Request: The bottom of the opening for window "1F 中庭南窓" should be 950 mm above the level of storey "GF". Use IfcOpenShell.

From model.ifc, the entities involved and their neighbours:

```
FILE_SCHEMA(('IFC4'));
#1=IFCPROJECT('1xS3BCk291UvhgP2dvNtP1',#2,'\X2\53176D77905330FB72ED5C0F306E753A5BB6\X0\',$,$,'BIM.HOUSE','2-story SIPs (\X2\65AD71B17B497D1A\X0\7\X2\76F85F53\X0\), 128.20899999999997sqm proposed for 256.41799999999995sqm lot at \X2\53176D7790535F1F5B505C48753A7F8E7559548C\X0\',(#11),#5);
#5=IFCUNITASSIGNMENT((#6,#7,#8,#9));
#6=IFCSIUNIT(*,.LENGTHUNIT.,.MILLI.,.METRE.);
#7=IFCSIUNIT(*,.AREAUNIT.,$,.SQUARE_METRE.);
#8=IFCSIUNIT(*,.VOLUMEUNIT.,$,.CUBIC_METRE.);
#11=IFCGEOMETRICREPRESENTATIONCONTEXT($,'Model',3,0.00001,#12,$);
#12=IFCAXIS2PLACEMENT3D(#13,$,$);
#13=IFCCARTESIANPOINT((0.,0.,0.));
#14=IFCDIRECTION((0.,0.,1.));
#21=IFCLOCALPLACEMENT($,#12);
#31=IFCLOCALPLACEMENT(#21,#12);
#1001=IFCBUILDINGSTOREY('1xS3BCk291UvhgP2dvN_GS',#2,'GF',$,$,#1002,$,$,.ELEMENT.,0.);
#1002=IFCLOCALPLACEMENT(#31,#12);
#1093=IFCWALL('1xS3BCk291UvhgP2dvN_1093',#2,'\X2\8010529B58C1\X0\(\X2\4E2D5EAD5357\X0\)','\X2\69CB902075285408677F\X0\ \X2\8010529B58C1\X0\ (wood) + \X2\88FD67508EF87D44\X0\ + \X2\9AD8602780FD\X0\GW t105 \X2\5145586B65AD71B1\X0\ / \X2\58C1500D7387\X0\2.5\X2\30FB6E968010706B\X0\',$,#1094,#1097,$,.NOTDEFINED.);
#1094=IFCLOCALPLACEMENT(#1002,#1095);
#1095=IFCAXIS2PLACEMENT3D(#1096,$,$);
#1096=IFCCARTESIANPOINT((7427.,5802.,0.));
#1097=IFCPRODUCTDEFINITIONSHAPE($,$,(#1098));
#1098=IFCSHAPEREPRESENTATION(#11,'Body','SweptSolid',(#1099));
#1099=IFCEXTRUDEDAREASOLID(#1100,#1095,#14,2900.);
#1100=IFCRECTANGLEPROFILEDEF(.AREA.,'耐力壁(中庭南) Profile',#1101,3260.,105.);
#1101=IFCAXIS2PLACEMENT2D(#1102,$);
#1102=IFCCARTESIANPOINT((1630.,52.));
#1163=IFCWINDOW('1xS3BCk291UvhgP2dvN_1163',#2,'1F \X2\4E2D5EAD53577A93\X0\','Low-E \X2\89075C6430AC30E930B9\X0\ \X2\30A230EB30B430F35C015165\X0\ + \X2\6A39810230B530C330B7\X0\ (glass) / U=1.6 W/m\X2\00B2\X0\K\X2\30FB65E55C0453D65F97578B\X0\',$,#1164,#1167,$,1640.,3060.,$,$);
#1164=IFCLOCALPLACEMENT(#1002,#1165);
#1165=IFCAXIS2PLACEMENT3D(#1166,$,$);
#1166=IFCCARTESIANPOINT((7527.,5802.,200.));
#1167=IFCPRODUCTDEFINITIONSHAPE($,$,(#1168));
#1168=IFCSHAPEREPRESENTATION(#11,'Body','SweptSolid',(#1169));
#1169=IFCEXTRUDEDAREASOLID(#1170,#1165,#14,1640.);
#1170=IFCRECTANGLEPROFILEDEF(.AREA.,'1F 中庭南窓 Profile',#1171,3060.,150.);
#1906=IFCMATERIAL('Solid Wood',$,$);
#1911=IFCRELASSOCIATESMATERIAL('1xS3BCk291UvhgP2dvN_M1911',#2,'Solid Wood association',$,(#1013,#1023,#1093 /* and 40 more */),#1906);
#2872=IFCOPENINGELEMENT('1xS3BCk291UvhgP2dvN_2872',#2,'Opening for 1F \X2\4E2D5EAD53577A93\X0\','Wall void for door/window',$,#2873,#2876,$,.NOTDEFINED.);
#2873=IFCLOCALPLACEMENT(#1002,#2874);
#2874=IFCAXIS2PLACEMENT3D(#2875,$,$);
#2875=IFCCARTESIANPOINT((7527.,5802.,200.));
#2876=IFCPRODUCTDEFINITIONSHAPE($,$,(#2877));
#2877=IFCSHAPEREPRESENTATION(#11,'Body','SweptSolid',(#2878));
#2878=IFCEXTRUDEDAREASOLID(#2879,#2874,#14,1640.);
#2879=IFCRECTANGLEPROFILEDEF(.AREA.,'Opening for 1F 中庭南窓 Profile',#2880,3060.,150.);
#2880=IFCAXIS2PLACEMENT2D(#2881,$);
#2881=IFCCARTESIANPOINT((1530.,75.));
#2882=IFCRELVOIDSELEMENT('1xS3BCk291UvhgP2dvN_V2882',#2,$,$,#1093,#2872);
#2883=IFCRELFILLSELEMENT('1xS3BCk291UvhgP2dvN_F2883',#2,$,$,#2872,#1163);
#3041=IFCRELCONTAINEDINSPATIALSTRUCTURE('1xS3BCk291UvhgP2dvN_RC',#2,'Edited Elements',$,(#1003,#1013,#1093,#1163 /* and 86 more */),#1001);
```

```python
import numpy as np
import ifcopenshell
import ifcopenshell.api.geometry
import ifcopenshell.geom
import ifcopenshell.util.element
import ifcopenshell.util.placement
import ifcopenshell.util.shape
import ifcopenshell.util.unit

model = ifcopenshell.open("model.ifc")
unit_scale = ifcopenshell.util.unit.calculate_unit_scale(model)

window = model.by_guid("1xS3BCk291UvhgP2dvN_1163")
opening = window.FillsVoids[0].RelatingOpeningElement
storey = ifcopenshell.util.element.get_container(window, ifc_class="IfcBuildingStorey")
level = ifcopenshell.util.placement.get_local_placement(storey.ObjectPlacement)[2, 3]

# The opening's origin need not be at the sill, so measure its lowest point.
shape = ifcopenshell.geom.create_shape(ifcopenshell.geom.settings(), opening)
bottom = ifcopenshell.util.shape.get_shape_bottom_elevation(shape, shape.geometry) / unit_scale
dz = level + 0.95 / unit_scale - bottom

shift = np.array([0.0, 0.0, dz])
# The window is not placed relative to its opening, so move both.
for product in (opening, window):
    matrix = ifcopenshell.util.placement.get_local_placement(product.ObjectPlacement)
    matrix[:3, 3] += shift
    ifcopenshell.api.geometry.edit_object_placement(model, product=product, matrix=matrix, is_si=False)

print(f"moved by {dz * unit_scale:+.3f} m")

model.write("model_v2.ifc")
```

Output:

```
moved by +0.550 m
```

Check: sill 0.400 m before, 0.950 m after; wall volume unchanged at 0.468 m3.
